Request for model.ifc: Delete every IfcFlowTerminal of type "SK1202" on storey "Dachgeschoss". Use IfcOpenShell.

First a look at what the model holds.

```python
import ifcopenshell
import ifcopenshell.util.element

model = ifcopenshell.open("model.ifc")
print(model.schema)
storey = next(s for s in model.by_type("IfcBuildingStorey") if s.Name == "Dachgeschoss")
terminals = [e for e in ifcopenshell.util.element.get_decomposition(storey) if e.is_a("IfcFlowTerminal")]
seen = {}
for e in terminals:
    element_type = ifcopenshell.util.element.get_type(e)
    name = element_type.Name if element_type not in (None, e) else None
    seen[name] = seen.get(name, 0) + 1
for name, count in sorted(seen.items(), key=str):
    print(count, "x", name)
```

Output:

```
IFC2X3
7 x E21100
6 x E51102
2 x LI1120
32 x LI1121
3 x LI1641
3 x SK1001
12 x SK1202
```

```python
import ifcopenshell
import ifcopenshell.api.root
import ifcopenshell.util.element

model = ifcopenshell.open("model.ifc")

storey = next(s for s in model.by_type("IfcBuildingStorey") if s.Name == "Dachgeschoss")
terminals = [e for e in ifcopenshell.util.element.get_decomposition(storey) if e.is_a("IfcFlowTerminal")]
targets = [e for e in terminals if (t := ifcopenshell.util.element.get_type(e)) not in (None, e) and t.Name == "SK1202"]

for e in targets:
    ifcopenshell.api.root.remove_product(model, product=e)
print(len(targets), "removed")

model.write("model_edited.ifc")
```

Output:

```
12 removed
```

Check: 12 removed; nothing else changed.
